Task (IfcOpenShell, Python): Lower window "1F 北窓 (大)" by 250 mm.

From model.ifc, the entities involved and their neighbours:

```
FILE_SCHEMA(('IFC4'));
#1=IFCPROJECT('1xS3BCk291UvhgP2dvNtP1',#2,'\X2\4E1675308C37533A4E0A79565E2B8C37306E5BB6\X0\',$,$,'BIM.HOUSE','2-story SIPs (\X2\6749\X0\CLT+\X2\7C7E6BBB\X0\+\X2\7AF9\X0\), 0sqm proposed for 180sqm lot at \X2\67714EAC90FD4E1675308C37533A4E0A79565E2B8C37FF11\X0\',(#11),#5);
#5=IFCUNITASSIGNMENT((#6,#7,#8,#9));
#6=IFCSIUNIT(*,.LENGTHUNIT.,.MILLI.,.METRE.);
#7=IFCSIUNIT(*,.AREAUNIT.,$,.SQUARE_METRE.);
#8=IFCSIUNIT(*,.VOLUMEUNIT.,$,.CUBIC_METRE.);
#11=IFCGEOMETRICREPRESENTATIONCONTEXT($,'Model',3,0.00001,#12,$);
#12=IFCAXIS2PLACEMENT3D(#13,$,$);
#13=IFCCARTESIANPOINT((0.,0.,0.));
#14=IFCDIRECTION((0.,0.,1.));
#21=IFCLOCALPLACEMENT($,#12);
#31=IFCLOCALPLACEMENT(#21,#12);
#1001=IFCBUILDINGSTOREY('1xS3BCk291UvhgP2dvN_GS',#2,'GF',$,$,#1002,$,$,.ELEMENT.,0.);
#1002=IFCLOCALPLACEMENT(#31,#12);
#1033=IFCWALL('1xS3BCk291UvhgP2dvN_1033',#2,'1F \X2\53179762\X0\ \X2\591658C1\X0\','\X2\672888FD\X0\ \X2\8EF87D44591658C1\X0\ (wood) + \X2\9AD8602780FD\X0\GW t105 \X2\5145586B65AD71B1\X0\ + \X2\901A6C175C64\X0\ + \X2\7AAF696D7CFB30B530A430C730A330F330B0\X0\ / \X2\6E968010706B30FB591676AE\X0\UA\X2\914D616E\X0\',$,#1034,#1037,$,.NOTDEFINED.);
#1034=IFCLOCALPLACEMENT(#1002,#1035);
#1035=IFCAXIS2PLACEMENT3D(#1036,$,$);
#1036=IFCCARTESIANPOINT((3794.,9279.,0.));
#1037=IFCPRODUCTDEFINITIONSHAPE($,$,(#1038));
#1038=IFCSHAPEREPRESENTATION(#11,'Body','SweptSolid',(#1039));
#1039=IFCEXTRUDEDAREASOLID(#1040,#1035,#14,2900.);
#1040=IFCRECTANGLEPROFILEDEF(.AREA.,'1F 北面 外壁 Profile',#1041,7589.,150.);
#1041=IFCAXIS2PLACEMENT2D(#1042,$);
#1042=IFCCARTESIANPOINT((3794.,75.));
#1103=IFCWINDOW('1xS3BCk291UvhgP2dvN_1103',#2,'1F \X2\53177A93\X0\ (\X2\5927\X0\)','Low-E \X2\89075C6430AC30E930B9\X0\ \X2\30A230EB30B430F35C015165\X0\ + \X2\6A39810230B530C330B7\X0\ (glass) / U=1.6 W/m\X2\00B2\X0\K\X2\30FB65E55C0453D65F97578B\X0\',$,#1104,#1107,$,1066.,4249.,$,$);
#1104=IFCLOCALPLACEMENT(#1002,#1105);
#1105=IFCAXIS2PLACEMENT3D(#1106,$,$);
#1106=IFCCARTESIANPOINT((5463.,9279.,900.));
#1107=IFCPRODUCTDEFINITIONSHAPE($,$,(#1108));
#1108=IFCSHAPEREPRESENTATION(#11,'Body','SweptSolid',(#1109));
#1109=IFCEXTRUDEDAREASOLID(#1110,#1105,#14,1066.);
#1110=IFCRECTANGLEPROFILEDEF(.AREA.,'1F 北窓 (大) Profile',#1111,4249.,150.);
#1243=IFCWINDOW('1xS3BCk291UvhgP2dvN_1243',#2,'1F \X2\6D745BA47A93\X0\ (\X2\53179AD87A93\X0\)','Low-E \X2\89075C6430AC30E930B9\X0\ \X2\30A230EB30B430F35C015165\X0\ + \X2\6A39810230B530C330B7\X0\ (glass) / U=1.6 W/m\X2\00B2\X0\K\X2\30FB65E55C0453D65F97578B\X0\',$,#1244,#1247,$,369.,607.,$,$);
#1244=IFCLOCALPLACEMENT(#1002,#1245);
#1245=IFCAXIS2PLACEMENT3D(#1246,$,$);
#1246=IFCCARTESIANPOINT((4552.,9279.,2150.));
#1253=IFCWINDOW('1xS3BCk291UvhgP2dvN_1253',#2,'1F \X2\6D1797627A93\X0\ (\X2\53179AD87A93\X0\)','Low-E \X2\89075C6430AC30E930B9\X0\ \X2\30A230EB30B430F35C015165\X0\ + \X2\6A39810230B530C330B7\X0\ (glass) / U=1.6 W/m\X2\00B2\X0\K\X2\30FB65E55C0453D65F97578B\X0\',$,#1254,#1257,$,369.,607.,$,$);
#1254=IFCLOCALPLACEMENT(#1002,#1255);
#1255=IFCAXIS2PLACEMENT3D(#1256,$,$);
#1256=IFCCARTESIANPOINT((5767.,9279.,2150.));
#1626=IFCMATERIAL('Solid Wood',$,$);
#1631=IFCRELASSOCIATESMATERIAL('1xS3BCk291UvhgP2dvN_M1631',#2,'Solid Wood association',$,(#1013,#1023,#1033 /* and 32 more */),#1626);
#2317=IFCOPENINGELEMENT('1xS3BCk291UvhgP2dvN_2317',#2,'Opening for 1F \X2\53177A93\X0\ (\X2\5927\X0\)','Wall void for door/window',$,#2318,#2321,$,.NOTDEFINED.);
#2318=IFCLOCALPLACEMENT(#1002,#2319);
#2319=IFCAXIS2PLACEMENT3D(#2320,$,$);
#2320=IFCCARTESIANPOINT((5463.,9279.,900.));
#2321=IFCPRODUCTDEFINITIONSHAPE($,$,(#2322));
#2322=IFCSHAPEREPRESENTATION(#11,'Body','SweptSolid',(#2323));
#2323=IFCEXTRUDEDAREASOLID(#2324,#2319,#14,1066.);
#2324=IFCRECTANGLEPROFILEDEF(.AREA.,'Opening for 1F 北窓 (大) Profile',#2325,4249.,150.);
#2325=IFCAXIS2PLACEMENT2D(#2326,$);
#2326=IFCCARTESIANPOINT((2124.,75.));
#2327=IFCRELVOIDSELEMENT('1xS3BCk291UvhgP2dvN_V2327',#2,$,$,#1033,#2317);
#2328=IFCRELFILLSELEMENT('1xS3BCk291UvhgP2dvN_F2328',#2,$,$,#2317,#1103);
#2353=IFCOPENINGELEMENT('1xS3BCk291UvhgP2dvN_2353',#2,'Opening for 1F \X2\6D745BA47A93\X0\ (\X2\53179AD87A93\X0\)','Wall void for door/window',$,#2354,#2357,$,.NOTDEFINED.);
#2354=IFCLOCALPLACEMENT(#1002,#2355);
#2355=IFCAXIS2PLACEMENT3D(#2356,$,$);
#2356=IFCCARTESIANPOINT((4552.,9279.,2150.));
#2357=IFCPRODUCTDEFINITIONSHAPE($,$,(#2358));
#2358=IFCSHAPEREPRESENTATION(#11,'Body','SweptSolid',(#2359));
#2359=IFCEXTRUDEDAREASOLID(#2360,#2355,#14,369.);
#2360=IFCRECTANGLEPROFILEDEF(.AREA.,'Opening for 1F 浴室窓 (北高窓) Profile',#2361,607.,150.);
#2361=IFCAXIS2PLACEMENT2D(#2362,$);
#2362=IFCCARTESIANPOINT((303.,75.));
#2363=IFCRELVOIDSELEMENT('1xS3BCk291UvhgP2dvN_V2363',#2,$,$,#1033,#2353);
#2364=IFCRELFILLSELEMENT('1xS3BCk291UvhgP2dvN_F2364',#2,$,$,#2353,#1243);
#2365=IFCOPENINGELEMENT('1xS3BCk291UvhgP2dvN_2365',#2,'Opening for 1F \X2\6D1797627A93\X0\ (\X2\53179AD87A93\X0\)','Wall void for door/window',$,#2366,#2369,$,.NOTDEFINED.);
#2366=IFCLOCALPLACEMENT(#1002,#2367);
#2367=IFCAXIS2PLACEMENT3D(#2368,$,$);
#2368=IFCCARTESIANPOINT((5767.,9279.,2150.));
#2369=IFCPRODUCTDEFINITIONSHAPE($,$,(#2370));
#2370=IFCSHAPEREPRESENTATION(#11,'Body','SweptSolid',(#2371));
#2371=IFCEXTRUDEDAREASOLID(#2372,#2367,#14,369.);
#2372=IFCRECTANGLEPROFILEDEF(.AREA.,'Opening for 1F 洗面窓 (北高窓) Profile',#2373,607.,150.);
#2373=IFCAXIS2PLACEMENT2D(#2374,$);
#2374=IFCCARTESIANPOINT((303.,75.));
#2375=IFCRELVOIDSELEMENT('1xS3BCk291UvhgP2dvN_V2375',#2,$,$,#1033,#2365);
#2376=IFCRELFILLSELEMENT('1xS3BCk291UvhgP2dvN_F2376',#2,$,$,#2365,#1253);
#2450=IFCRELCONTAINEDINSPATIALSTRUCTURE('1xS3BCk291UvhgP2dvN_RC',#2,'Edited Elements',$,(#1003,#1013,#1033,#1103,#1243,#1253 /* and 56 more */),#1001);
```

```python
import numpy as np
import ifcopenshell
import ifcopenshell.api.geometry
import ifcopenshell.util.placement
import ifcopenshell.util.unit

model = ifcopenshell.open("model.ifc")
unit_scale = ifcopenshell.util.unit.calculate_unit_scale(model)

window = model.by_id(1103)
opening = window.FillsVoids[0].RelatingOpeningElement
dz = -0.25 / unit_scale

shift = np.array([0.0, 0.0, dz])
# The window is not placed relative to its opening, so move both.
for product in (opening, window):
    matrix = ifcopenshell.util.placement.get_local_placement(product.ObjectPlacement)
    matrix[:3, 3] += shift
    ifcopenshell.api.geometry.edit_object_placement(model, product=product, matrix=matrix, is_si=False)

print(f"moved by {dz * unit_scale:+.3f} m")

model.write("model_v2.ifc")
```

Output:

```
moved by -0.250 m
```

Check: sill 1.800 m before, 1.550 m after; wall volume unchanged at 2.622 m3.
